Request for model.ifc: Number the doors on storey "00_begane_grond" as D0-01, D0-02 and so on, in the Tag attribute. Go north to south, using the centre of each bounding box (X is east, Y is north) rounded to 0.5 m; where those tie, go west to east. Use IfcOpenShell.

First a look at what the model holds.

```python
import ifcopenshell
import ifcopenshell.util.element
import ifcopenshell.util.placement

model = ifcopenshell.open("model.ifc")
print(model.schema)
storey = next(s for s in model.by_type("IfcBuildingStorey") if s.Name == "00_begane_grond")
doors = [e for e in ifcopenshell.util.element.get_decomposition(storey) if e.is_a("IfcDoor")]
for e in sorted(doors, key=lambda e: e.id()):
    origin = ifcopenshell.util.placement.get_local_placement(e.ObjectPlacement)[:3, 3]
    print(e.id(), e.Tag, e.Name, origin.round(2) + 0.0, sep=" | ")
```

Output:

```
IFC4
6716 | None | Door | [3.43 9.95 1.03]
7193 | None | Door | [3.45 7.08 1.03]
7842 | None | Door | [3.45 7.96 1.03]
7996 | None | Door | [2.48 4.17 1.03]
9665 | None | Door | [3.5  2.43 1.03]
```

```python
import ifcopenshell
import ifcopenshell.geom
import ifcopenshell.util.element
import ifcopenshell.util.shape

model = ifcopenshell.open("model.ifc")
settings = ifcopenshell.geom.settings()
settings.set("use-world-coords", True)


def centre(element):
    shape = ifcopenshell.geom.create_shape(settings, element)
    return ifcopenshell.util.shape.get_bbox_centroid(shape.geometry)


storey = next(s for s in model.by_type("IfcBuildingStorey") if s.Name == "00_begane_grond")
doors = [e for e in ifcopenshell.util.element.get_decomposition(storey) if e.is_a("IfcDoor")]

# Insertion points can sit at a corner or the storey origin, so sort by the geometry (in metres).
centres = {e: centre(e) for e in doors}
doors.sort(key=lambda e: (-round(centres[e][1] / 0.5), centres[e][0]))

for i, e in enumerate(doors, start=1):
    number = f"D0-{i:02d}"
    e.Tag = number
    print(e.id(), number)

model.write("model_v2.ifc")
```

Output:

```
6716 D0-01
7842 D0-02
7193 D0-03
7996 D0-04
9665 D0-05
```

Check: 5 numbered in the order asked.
